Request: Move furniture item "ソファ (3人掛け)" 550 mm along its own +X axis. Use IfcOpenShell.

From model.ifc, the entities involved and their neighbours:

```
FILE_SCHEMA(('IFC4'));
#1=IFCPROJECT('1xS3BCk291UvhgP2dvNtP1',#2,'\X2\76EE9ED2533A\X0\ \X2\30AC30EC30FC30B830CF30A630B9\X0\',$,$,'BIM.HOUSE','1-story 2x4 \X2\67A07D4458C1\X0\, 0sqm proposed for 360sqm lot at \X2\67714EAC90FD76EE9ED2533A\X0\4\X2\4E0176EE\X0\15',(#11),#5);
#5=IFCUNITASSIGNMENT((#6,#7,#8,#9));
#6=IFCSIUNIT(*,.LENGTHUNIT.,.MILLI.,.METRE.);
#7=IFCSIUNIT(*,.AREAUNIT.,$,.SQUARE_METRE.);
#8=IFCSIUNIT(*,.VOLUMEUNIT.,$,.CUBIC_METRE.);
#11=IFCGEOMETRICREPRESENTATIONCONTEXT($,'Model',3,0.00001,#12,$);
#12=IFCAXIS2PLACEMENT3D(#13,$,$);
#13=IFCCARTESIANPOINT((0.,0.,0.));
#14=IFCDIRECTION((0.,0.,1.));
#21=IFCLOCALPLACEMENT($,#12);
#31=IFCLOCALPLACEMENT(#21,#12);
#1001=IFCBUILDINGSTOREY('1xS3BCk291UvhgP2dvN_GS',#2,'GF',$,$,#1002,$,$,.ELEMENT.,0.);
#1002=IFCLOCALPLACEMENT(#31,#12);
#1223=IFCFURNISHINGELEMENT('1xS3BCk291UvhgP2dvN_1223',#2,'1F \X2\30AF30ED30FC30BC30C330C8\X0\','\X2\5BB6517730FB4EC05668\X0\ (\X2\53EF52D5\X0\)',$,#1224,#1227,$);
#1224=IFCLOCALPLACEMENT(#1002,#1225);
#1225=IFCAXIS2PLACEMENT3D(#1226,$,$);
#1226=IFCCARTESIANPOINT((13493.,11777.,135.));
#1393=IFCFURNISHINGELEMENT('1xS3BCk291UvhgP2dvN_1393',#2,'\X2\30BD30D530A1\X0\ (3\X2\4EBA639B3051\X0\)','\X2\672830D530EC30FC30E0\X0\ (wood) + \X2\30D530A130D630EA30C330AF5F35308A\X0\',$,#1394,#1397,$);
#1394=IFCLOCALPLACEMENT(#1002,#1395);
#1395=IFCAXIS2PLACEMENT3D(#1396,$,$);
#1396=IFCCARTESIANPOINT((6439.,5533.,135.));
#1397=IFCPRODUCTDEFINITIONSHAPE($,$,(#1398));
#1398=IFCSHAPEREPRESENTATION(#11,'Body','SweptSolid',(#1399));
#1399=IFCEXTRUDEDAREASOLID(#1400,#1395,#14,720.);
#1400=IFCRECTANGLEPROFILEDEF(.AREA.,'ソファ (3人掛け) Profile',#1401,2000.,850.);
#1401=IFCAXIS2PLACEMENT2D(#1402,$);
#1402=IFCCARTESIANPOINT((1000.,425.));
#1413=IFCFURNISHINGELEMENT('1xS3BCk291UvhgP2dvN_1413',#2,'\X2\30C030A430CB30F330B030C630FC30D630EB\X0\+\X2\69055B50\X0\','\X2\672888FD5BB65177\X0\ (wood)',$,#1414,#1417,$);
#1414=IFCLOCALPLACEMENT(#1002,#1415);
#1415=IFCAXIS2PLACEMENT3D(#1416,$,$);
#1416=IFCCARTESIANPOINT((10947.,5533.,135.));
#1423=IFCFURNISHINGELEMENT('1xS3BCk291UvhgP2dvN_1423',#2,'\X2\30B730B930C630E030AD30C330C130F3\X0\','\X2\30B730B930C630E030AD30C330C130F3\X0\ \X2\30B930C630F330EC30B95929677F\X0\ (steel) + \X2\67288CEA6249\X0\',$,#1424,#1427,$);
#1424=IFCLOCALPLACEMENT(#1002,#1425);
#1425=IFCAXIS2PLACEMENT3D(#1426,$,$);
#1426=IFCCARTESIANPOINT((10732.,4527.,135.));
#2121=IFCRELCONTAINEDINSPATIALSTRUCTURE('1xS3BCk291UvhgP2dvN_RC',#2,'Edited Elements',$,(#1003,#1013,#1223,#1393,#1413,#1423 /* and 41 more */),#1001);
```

```python
import ifcopenshell
import ifcopenshell.api.geometry
import ifcopenshell.util.placement

model = ifcopenshell.open("model.ifc")

item = model.by_guid("1xS3BCk291UvhgP2dvN_1393")
matrix = ifcopenshell.util.placement.get_local_placement(item.ObjectPlacement)
matrix[:3, 3] += matrix[:3, 0] * 550.0
ifcopenshell.api.geometry.edit_object_placement(model, product=item, matrix=matrix, is_si=False)

print(ifcopenshell.util.placement.get_local_placement(item.ObjectPlacement).round(3) + 0.0)

model.write("model_rev.ifc")
```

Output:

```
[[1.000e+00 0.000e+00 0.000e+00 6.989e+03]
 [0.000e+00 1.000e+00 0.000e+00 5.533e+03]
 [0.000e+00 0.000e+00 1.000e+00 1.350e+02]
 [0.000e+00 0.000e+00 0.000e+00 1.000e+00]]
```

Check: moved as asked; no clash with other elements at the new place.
